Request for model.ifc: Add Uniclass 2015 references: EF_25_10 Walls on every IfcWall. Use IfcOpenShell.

First a look at what the model holds.

```python
import ifcopenshell

model = ifcopenshell.open("model.ifc")
print(model.schema)
print("classifications:", [c.Name for c in model.by_type("IfcClassification")])
for ifc_class in ("IfcDoor", "IfcRoof", "IfcStair", "IfcWall", "IfcWindow"):
    print(ifc_class, len(model.by_type(ifc_class)))
```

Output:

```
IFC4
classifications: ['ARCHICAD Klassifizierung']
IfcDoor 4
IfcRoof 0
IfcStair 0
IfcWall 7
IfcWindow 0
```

```python
import ifcopenshell
import ifcopenshell.api.classification

model = ifcopenshell.open("model.ifc")

system = ifcopenshell.api.classification.add_classification(model, classification="Uniclass 2015")

codes = {
    "IfcWall": ("EF_25_10", "Walls"),
}
for ifc_class, (code, name) in codes.items():
    products = model.by_type(ifc_class)
    ifcopenshell.api.classification.add_reference(
        model, products=products, classification=system, identification=code, name=name
    )
    print(code, len(products))

model.write("model_rev.ifc")
```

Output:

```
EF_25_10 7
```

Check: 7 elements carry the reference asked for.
